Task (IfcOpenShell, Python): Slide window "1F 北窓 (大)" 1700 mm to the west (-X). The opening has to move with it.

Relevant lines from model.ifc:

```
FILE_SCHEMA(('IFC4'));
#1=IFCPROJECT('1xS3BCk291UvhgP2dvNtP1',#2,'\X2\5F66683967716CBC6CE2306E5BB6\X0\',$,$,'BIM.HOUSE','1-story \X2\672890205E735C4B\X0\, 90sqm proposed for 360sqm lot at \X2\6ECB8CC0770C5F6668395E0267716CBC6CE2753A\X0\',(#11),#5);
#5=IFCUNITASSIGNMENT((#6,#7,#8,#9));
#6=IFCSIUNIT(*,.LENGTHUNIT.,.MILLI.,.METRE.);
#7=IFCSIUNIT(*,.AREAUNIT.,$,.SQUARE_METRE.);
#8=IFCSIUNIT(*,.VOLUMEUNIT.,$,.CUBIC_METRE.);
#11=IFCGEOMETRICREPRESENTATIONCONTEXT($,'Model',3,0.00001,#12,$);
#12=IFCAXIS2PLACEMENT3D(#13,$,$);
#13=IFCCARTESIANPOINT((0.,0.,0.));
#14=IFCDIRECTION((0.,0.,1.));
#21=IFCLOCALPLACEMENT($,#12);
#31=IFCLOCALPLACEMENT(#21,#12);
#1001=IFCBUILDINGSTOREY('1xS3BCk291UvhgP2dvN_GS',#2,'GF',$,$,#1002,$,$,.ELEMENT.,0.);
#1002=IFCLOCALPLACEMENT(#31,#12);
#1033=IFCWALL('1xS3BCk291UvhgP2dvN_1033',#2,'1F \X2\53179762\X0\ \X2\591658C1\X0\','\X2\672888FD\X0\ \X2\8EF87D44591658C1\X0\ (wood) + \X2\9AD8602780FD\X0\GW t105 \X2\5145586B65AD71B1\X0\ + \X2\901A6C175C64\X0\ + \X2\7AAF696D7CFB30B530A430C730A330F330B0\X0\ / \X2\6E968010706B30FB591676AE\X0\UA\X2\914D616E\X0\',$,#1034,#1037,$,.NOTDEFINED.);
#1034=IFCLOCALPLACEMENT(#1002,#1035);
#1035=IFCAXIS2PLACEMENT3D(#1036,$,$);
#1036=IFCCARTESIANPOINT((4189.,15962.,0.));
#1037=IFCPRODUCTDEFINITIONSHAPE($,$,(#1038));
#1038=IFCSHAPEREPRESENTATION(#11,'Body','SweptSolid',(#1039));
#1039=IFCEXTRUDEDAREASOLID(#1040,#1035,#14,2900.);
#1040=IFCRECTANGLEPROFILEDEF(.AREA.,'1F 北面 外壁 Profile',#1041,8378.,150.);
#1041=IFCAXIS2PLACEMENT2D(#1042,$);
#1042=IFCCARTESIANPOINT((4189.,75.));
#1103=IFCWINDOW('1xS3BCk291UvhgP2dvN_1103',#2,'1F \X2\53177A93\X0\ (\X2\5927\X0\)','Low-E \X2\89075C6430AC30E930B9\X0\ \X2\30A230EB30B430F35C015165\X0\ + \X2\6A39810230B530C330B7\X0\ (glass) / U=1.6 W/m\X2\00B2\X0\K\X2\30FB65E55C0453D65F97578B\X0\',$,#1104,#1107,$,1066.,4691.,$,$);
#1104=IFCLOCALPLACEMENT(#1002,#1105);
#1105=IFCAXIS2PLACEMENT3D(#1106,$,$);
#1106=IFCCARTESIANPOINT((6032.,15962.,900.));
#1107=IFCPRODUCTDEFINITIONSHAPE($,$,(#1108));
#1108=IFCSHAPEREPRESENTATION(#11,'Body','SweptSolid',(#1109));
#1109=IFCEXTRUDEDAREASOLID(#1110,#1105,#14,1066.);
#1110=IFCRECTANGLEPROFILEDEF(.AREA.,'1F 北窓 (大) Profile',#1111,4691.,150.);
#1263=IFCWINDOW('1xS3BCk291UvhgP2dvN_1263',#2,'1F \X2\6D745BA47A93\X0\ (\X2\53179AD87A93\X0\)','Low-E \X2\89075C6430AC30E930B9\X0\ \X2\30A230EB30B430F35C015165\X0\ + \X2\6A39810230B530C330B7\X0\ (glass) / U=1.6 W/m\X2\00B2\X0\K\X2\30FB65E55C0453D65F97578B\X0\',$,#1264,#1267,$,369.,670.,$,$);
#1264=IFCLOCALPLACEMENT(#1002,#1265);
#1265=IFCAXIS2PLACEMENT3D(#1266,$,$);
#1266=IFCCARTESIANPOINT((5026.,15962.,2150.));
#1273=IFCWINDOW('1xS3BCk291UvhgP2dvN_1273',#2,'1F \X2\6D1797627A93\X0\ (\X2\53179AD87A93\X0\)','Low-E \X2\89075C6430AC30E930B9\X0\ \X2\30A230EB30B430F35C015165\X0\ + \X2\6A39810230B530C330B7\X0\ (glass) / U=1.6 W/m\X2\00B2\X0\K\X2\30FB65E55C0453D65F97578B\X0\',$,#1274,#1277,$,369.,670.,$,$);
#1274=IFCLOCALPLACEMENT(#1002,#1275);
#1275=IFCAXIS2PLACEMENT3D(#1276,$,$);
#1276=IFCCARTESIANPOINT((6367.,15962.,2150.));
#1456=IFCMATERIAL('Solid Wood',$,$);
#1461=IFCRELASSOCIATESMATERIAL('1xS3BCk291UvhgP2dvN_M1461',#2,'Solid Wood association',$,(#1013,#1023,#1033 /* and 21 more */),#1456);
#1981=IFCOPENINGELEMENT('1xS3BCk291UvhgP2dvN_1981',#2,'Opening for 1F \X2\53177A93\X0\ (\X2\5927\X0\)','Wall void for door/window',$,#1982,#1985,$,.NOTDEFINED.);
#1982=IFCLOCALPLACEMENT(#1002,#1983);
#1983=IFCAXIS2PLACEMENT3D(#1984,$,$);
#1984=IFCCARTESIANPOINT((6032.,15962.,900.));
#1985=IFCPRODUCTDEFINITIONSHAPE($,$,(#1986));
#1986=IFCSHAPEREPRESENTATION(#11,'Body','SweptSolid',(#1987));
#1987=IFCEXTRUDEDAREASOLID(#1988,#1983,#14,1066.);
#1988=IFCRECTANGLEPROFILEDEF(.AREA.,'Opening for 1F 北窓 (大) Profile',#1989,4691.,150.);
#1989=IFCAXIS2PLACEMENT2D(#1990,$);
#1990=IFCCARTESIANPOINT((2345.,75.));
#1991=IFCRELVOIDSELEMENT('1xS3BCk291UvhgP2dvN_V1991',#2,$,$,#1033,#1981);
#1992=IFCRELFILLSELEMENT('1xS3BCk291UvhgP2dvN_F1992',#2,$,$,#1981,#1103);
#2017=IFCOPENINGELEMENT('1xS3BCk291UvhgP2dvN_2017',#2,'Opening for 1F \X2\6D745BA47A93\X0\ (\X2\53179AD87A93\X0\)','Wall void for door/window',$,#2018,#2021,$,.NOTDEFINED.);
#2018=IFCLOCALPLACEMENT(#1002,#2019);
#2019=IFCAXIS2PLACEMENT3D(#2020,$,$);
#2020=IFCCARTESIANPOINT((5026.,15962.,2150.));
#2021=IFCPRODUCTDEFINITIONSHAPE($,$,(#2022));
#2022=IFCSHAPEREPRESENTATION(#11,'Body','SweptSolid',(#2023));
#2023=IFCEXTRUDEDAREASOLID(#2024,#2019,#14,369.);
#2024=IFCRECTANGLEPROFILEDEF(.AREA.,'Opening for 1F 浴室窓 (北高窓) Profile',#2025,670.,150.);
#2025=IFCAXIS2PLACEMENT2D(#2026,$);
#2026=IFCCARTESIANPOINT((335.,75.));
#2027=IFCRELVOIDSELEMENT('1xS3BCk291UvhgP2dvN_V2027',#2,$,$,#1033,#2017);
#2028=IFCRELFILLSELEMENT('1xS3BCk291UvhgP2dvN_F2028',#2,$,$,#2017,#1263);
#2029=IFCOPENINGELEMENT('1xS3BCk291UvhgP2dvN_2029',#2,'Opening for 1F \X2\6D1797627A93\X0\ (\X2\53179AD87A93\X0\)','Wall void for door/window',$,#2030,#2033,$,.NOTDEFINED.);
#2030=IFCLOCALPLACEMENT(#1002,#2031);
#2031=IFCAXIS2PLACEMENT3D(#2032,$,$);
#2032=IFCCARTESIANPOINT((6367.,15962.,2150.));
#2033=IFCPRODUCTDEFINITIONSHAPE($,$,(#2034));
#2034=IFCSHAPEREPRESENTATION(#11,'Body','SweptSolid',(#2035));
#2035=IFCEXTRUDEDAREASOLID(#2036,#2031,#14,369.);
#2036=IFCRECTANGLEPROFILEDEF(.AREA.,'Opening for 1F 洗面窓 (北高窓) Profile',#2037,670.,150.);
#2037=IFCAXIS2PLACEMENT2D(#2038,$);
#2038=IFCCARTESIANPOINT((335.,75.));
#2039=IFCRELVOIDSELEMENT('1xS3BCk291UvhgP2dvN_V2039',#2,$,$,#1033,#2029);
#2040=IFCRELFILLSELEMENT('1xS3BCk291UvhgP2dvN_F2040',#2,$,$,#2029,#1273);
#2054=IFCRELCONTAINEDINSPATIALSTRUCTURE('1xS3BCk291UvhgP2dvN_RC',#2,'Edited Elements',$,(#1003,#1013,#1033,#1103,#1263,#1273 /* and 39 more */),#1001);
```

```python
import ifcopenshell
import ifcopenshell.api.geometry
import ifcopenshell.util.placement
import ifcopenshell.util.unit

model = ifcopenshell.open("model.ifc")
unit_scale = ifcopenshell.util.unit.calculate_unit_scale(model)

window = model.by_id(1103)
opening = window.FillsVoids[0].RelatingOpeningElement
wall = opening.VoidsElements[0].RelatingBuildingElement

wall_matrix = ifcopenshell.util.placement.get_local_placement(wall.ObjectPlacement)
shift = wall_matrix[:3, 0] * -1.7 / unit_scale
before = ifcopenshell.util.placement.get_local_placement(window.ObjectPlacement)[:3, 3].copy()

# The window is not placed relative to its opening, so move both.
for product in (opening, window):
    matrix = ifcopenshell.util.placement.get_local_placement(product.ObjectPlacement)
    matrix[:3, 3] += shift
    ifcopenshell.api.geometry.edit_object_placement(model, product=product, matrix=matrix, is_si=False)

after = ifcopenshell.util.placement.get_local_placement(window.ObjectPlacement)[:3, 3]
print("window moved by", (after - before).round(3) + 0.0)

model.write("model_edited.ifc")
```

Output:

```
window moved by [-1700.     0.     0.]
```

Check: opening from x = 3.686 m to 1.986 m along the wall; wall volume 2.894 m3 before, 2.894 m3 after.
